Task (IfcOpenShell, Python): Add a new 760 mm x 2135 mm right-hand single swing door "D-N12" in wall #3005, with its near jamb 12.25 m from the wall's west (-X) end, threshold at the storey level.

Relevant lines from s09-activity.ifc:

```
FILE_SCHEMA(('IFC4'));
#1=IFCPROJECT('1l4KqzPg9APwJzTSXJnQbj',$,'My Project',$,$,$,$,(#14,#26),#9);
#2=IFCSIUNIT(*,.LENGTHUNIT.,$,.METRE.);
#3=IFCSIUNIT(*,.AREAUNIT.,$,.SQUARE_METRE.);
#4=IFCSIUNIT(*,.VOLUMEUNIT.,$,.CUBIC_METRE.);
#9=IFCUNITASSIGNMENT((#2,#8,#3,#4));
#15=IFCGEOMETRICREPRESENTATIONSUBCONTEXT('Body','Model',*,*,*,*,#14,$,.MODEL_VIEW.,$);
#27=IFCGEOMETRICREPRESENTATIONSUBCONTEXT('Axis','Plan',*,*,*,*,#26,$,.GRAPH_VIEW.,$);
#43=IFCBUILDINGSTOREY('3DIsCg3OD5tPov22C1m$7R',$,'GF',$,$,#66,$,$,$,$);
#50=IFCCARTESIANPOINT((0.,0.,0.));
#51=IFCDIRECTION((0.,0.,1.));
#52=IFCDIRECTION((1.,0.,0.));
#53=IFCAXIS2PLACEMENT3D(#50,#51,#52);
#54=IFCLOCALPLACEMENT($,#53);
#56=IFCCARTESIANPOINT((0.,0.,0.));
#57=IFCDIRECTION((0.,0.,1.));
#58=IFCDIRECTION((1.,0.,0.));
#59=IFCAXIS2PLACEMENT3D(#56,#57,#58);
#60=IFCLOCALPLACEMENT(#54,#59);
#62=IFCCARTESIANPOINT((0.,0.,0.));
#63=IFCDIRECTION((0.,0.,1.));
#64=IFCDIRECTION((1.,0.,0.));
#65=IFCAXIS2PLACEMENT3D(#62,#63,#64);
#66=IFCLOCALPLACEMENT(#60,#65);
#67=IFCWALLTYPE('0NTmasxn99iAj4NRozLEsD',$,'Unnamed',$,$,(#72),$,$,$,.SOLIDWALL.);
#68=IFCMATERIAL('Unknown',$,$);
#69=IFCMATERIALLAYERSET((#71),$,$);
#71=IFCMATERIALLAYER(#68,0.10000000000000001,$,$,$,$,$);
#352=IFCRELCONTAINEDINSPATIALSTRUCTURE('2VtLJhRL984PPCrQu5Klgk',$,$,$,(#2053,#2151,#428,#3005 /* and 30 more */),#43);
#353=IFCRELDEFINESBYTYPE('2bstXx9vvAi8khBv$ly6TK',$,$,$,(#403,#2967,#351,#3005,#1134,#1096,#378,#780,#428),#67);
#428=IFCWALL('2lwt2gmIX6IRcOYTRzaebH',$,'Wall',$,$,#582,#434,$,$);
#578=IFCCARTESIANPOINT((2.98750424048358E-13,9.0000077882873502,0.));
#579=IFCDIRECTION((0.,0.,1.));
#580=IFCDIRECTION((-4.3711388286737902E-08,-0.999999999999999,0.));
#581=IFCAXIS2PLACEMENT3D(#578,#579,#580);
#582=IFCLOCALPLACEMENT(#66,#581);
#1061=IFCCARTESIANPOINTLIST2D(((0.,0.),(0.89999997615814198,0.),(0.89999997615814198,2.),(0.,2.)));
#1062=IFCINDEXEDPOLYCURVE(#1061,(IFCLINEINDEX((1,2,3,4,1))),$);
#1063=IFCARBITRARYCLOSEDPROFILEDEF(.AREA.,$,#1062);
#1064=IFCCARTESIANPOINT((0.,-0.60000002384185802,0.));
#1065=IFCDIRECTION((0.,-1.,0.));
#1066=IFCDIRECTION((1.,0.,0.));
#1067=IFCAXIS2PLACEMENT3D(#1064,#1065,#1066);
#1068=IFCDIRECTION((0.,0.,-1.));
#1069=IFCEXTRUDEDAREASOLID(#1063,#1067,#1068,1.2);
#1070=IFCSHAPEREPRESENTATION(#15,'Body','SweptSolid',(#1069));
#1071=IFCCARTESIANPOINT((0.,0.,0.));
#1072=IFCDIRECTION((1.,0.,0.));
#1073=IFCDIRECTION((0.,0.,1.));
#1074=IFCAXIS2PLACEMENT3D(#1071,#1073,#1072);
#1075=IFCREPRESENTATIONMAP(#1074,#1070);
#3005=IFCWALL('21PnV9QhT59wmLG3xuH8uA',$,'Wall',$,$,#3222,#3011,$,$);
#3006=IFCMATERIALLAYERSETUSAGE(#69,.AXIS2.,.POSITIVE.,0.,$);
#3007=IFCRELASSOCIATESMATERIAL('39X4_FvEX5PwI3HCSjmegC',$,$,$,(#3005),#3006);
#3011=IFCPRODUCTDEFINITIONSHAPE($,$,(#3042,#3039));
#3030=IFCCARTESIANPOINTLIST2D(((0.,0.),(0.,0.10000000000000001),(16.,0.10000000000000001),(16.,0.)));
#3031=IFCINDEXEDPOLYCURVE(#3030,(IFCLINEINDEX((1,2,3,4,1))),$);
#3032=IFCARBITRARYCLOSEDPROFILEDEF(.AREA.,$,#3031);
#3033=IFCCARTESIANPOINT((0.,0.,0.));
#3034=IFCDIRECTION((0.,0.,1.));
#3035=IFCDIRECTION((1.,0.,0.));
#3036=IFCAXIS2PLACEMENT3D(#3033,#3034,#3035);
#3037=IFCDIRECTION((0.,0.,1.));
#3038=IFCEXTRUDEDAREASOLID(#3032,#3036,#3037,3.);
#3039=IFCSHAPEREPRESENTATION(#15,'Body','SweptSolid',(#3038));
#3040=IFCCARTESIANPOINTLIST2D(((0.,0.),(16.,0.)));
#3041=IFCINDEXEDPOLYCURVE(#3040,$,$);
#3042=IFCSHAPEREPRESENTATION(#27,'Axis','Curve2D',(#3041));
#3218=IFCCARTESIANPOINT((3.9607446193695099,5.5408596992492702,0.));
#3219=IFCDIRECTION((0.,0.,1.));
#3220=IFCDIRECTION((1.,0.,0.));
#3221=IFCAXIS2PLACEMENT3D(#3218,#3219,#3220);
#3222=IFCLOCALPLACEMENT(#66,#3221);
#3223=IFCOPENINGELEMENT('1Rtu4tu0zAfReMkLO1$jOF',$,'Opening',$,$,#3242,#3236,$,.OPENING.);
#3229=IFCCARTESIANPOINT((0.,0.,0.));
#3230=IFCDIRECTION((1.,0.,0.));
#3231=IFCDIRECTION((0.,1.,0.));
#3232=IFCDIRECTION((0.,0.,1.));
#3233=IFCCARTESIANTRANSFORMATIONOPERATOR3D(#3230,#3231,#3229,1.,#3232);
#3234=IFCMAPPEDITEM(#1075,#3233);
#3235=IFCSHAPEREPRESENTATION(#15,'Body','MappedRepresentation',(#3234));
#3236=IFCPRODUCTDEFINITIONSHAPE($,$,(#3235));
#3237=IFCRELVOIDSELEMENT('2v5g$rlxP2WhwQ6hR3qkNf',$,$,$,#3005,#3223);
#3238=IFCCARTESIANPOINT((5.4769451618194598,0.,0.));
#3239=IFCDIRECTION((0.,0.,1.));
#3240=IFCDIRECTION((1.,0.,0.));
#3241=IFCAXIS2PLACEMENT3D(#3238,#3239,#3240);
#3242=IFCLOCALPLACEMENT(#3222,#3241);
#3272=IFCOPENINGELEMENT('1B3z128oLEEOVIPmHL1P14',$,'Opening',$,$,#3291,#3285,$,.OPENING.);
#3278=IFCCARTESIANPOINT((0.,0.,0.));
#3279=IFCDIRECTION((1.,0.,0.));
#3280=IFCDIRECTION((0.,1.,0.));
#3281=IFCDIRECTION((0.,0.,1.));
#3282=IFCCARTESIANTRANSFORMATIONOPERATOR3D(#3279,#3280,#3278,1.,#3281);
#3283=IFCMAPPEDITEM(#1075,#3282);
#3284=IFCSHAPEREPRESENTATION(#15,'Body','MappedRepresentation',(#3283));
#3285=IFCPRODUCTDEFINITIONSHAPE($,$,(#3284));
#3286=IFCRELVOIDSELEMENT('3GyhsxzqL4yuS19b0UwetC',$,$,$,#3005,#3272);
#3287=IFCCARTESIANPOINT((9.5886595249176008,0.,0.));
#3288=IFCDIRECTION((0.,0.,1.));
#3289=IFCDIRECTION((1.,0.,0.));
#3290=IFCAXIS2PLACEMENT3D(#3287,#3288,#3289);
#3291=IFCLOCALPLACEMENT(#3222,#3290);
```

```python
import numpy as np
import ifcopenshell
import ifcopenshell.api.feature
import ifcopenshell.api.geometry
import ifcopenshell.api.root
import ifcopenshell.api.spatial
import ifcopenshell.geom
import ifcopenshell.util.element
import ifcopenshell.util.placement
import ifcopenshell.util.representation
import ifcopenshell.util.shape
import ifcopenshell.util.unit

model = ifcopenshell.open("s09-activity.ifc")
unit_scale = ifcopenshell.util.unit.calculate_unit_scale(model)
settings = ifcopenshell.geom.settings()


def volume(element):
    """Net volume in cubic metres, openings subtracted."""
    shape = ifcopenshell.geom.create_shape(settings, element)
    return ifcopenshell.util.shape.get_volume(shape.geometry)


wall = model.by_id(3005)
storey = ifcopenshell.util.element.get_container(wall, ifc_class="IfcBuildingStorey")
context = ifcopenshell.util.representation.get_context(model, "Model", "Body", "MODEL_VIEW")
before = volume(wall)

width, height, from_end, sill = 0.76, 2.135, 12.25, 0.0  # metres

# The wall runs along its own X axis, and the end named is its -X end.
wall_shape = ifcopenshell.geom.create_shape(settings, wall)
x, y, z = ifcopenshell.util.shape.get_vertices(wall_shape.geometry).T
start = x.min() + from_end
face, thickness = float(y.min()), float(y.max() - y.min())
wall_matrix = ifcopenshell.util.placement.get_local_placement(wall.ObjectPlacement)
level = ifcopenshell.util.placement.get_local_placement(storey.ObjectPlacement)[2, 3]


def in_wall(x, y):
    """Placement at x, y metres in the wall's axes, at sill height."""
    matrix = wall_matrix.copy()
    matrix[:, 3] = wall_matrix @ np.array([x / unit_scale, y / unit_scale, 0.0, 1.0])
    matrix[2, 3] = level + sill / unit_scale
    return matrix


# Opening: a box that overshoots both wall faces by 50 mm.
opening = ifcopenshell.api.root.create_entity(model, ifc_class="IfcOpeningElement", predefined_type="OPENING")
box = ifcopenshell.api.geometry.add_wall_representation(
    model, context=context, length=width, height=height, thickness=thickness + 0.1
)
ifcopenshell.api.geometry.assign_representation(model, product=opening, representation=box)
ifcopenshell.api.geometry.edit_object_placement(model, product=opening, matrix=in_wall(start, face - 0.05), is_si=False)
ifcopenshell.api.feature.add_feature(model, feature=opening, element=wall)

door = ifcopenshell.api.root.create_entity(model, ifc_class="IfcDoor", name="D-N12", predefined_type="DOOR")
door.OverallWidth, door.OverallHeight = width / unit_scale, height / unit_scale
door.OperationType = "SINGLE_SWING_RIGHT"
body = ifcopenshell.api.geometry.add_door_representation(
    model,
    context=context,
    overall_width=door.OverallWidth,
    overall_height=door.OverallHeight,
    operation_type="SINGLE_SWING_RIGHT",
    lining_properties={"LiningDepth": thickness / unit_scale, "ThresholdDepth": thickness / unit_scale},
)
ifcopenshell.api.geometry.assign_representation(model, product=door, representation=body)
ifcopenshell.api.spatial.assign_container(model, products=[door], relating_structure=storey)
ifcopenshell.api.feature.add_filling(model, opening=opening, element=door)

# The lining spans the wall, so the door starts at the wall face.
ifcopenshell.api.geometry.edit_object_placement(model, product=door, matrix=in_wall(start, face), is_si=False)

after = volume(wall)

print(f"wall volume {before:.3f} -> {after:.3f} m3")

model.write("s09-activity_rev.ifc")
```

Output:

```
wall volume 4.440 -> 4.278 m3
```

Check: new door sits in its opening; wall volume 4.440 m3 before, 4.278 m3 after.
